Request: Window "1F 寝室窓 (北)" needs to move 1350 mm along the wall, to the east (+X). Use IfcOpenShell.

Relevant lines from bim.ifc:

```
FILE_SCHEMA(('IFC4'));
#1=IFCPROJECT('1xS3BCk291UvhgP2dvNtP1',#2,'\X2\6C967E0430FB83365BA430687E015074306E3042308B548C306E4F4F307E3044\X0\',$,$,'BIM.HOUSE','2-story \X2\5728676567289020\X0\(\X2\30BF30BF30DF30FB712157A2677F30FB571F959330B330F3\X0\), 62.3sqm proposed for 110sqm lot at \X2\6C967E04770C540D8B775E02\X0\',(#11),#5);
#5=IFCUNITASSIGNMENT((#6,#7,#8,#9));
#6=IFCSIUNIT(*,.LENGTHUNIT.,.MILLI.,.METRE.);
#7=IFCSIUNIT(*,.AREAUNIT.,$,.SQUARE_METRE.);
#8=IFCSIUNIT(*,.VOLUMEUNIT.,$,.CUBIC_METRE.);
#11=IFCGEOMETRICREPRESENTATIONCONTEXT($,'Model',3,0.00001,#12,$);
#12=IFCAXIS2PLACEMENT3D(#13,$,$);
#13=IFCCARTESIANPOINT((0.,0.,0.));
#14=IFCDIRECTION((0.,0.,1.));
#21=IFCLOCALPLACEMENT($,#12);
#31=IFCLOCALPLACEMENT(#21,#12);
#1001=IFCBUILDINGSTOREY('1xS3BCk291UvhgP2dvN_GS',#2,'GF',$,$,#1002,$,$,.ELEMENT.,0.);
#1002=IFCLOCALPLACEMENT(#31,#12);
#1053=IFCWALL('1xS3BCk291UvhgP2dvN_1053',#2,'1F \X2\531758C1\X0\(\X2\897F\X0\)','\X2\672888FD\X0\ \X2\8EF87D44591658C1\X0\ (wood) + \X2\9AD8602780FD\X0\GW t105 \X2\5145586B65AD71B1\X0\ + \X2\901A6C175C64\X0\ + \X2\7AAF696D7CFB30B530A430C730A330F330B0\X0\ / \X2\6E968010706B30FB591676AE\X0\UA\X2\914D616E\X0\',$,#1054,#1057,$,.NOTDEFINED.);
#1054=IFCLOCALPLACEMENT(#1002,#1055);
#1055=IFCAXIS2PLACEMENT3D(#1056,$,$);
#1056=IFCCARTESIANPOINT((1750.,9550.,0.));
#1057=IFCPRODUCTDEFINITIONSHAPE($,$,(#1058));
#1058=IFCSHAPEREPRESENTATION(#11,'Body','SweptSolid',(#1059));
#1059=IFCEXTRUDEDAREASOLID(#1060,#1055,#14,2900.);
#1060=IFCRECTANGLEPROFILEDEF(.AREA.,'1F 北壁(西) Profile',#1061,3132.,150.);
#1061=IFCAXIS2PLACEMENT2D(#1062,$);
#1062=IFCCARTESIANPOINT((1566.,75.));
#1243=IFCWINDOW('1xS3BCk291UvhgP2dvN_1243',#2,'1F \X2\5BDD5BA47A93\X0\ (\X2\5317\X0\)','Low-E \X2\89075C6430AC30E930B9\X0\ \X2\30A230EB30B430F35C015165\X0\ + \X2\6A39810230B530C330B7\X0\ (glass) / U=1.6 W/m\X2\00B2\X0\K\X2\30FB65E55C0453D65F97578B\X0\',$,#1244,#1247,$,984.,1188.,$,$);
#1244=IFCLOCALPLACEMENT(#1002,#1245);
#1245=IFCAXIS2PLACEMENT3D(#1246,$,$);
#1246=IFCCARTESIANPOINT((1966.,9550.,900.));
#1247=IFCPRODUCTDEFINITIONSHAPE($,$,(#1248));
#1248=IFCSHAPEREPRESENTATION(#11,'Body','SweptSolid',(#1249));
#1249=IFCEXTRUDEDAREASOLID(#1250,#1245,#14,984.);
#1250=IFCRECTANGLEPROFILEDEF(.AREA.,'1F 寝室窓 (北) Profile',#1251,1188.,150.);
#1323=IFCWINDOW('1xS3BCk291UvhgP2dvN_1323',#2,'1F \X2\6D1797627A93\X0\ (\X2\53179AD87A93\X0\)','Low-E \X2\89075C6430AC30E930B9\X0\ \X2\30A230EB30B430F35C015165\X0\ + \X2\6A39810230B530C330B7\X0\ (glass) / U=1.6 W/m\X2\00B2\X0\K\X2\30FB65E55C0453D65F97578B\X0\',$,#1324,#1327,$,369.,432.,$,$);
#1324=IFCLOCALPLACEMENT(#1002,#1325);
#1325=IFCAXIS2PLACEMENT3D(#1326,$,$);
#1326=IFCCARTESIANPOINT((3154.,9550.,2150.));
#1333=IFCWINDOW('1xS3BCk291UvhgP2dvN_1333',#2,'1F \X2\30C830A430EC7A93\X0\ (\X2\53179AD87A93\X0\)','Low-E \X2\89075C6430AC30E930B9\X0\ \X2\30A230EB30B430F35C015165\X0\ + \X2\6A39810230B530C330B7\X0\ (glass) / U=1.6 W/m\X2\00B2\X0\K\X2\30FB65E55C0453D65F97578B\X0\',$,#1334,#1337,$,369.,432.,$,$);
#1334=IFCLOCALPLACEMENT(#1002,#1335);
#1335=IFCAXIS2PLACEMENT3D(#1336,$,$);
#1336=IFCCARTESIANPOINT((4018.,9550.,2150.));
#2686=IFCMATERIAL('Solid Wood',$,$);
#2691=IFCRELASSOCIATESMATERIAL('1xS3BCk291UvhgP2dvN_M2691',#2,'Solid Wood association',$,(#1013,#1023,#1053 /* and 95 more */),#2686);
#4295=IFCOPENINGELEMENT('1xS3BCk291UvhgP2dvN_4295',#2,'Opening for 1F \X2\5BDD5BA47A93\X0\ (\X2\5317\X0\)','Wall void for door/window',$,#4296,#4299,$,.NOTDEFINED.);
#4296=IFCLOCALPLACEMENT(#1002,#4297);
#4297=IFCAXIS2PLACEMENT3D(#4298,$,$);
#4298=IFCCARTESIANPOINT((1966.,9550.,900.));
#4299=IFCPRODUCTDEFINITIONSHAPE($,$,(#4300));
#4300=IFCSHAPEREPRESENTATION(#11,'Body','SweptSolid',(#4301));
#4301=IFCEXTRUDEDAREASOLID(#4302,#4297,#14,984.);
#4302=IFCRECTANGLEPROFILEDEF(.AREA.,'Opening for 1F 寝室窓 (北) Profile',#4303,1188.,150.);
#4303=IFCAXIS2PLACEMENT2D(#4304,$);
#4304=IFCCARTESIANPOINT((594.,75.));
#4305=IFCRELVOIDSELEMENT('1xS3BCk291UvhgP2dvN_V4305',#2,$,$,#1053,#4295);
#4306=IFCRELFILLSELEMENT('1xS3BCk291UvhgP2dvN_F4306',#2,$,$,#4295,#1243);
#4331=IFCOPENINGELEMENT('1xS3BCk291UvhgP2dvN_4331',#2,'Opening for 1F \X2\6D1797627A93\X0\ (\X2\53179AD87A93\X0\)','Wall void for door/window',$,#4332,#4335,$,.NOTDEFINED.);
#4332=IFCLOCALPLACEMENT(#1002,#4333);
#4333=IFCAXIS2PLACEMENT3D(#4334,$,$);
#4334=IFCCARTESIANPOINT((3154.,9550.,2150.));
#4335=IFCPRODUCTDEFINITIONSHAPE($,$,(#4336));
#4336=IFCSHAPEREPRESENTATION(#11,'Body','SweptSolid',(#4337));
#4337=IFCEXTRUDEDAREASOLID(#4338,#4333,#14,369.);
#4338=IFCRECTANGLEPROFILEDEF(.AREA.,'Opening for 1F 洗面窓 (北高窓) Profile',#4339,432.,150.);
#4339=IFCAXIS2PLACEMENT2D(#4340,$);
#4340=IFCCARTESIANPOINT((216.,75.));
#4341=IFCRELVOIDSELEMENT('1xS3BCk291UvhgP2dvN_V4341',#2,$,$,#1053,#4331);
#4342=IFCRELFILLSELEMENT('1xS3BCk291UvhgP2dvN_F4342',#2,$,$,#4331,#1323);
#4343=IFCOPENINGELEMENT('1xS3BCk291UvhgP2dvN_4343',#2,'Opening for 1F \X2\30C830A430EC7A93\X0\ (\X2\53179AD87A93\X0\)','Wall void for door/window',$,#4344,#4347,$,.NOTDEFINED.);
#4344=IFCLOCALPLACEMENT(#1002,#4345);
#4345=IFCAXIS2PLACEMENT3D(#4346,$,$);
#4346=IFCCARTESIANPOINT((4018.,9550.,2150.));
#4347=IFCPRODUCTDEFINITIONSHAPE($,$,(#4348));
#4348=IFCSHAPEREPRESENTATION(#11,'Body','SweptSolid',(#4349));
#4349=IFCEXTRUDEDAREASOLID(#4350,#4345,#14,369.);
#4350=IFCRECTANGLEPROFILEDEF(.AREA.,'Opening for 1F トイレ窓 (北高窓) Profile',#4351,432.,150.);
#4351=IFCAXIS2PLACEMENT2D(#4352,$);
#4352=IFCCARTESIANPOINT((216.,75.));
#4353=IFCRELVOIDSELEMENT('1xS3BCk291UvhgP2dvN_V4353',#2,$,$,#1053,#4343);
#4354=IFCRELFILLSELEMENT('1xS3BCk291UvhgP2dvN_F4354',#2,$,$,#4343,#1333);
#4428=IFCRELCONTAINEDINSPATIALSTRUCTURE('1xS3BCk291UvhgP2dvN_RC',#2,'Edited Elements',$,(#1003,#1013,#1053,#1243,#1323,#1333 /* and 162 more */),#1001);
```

```python
import ifcopenshell
import ifcopenshell.api.geometry
import ifcopenshell.util.placement
import ifcopenshell.util.unit

model = ifcopenshell.open("bim.ifc")
unit_scale = ifcopenshell.util.unit.calculate_unit_scale(model)

window = model.by_guid("1xS3BCk291UvhgP2dvN_1243")
opening = window.FillsVoids[0].RelatingOpeningElement
wall = opening.VoidsElements[0].RelatingBuildingElement

wall_matrix = ifcopenshell.util.placement.get_local_placement(wall.ObjectPlacement)
shift = wall_matrix[:3, 0] * 1.35 / unit_scale
before = ifcopenshell.util.placement.get_local_placement(window.ObjectPlacement)[:3, 3].copy()

# The window is not placed relative to its opening, so move both.
for product in (opening, window):
    matrix = ifcopenshell.util.placement.get_local_placement(product.ObjectPlacement)
    matrix[:3, 3] += shift
    ifcopenshell.api.geometry.edit_object_placement(model, product=product, matrix=matrix, is_si=False)

after = ifcopenshell.util.placement.get_local_placement(window.ObjectPlacement)[:3, 3]
print("window moved by", (after - before).round(3) + 0.0)

model.write("bim_edited.ifc")
```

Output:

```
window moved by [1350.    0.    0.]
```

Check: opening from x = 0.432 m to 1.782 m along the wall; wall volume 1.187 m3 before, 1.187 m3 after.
